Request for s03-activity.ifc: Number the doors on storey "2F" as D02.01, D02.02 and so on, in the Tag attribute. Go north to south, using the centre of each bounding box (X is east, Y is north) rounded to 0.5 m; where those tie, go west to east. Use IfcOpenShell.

First a look at what the model holds.

```python
import ifcopenshell
import ifcopenshell.util.element
import ifcopenshell.util.placement

model = ifcopenshell.open("s03-activity.ifc")
print(model.schema)
storey = next(s for s in model.by_type("IfcBuildingStorey") if s.Name == "2F")
doors = [e for e in ifcopenshell.util.element.get_decomposition(storey) if e.is_a("IfcDoor")]
for e in sorted(doors, key=lambda e: e.id()):
    origin = ifcopenshell.util.placement.get_local_placement(e.ObjectPlacement)[:3, 3]
    print(e.id(), e.Tag, e.Name, origin.round(2) + 0.0, sep=" | ")
```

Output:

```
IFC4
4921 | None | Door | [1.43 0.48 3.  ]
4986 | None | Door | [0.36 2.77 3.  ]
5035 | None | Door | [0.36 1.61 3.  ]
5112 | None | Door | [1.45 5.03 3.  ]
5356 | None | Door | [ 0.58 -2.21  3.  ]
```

```python
import ifcopenshell
import ifcopenshell.geom
import ifcopenshell.util.element
import ifcopenshell.util.shape

model = ifcopenshell.open("s03-activity.ifc")
settings = ifcopenshell.geom.settings()
settings.set("use-world-coords", True)


def centre(element):
    shape = ifcopenshell.geom.create_shape(settings, element)
    return ifcopenshell.util.shape.get_bbox_centroid(shape.geometry)


storey = next(s for s in model.by_type("IfcBuildingStorey") if s.Name == "2F")
doors = [e for e in ifcopenshell.util.element.get_decomposition(storey) if e.is_a("IfcDoor")]

# Insertion points can sit at a corner or the storey origin, so sort by the geometry (in metres).
centres = {e: centre(e) for e in doors}
doors.sort(key=lambda e: (-round(centres[e][1] / 0.5), centres[e][0]))

for i, e in enumerate(doors, start=1):
    number = f"D02.{i:02d}"
    e.Tag = number
    print(e.id(), number)

model.write("s03-activity-out.ifc")
```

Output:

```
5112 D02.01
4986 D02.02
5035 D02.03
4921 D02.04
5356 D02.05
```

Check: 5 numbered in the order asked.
